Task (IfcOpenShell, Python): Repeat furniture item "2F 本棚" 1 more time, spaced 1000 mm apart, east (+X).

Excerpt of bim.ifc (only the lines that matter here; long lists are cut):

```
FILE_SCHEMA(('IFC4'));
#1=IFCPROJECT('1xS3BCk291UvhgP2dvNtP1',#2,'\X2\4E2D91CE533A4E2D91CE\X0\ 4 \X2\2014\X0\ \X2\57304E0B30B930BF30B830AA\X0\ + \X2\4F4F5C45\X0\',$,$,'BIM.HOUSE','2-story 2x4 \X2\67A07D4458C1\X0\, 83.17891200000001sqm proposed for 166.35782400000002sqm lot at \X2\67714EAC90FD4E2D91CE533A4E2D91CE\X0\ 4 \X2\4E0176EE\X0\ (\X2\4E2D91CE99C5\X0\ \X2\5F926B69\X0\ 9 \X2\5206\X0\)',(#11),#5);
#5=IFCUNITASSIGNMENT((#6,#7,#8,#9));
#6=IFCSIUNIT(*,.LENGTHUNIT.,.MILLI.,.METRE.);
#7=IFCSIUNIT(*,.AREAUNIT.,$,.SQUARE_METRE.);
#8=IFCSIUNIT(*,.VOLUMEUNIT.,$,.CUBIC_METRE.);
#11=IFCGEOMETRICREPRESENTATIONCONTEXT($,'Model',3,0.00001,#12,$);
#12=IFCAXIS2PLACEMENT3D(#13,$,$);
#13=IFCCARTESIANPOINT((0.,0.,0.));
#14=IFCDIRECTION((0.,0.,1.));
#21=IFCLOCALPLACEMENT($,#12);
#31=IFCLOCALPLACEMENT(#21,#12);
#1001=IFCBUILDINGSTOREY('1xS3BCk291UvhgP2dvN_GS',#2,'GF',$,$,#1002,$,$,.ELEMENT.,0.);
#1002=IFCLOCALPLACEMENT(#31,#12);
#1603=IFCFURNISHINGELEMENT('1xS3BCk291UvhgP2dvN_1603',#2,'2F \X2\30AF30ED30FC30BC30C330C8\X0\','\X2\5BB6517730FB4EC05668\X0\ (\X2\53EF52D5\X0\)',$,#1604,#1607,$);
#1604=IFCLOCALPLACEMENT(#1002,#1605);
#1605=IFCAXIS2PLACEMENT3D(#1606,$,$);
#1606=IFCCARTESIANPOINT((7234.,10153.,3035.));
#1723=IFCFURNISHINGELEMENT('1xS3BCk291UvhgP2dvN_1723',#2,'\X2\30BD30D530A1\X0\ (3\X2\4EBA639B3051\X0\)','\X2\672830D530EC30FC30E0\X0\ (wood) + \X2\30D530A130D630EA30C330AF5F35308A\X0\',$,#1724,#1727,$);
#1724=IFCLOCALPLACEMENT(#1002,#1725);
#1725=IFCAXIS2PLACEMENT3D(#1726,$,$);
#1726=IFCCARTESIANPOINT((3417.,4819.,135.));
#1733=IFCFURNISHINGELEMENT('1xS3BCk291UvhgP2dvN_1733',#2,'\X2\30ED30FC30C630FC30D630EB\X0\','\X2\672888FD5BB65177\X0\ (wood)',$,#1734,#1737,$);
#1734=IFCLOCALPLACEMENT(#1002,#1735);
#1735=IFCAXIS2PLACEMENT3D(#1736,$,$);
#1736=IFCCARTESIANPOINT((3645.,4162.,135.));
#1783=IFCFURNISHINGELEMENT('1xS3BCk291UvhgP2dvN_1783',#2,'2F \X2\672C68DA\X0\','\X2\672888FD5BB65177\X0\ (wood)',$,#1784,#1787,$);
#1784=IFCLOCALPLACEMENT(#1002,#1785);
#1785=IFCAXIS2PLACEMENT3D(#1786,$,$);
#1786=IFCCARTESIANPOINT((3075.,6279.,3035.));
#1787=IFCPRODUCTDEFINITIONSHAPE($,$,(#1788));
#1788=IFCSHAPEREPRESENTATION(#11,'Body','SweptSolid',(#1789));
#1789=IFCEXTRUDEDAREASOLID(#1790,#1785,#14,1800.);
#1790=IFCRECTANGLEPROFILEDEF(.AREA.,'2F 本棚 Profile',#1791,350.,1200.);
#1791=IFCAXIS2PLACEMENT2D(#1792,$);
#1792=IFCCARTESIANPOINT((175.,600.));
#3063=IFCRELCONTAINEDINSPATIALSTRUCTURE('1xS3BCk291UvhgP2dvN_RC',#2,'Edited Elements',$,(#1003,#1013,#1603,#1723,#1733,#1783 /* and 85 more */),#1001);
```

```python
import numpy as np
import ifcopenshell
import ifcopenshell.api.geometry
import ifcopenshell.api.root
import ifcopenshell.util.element
import ifcopenshell.util.placement
import ifcopenshell.util.unit

model = ifcopenshell.open("bim.ifc")
unit_scale = ifcopenshell.util.unit.calculate_unit_scale(model)


def reuse_history(source, copy):
    """copy_class also copies each property set's owner history, people and application; keep the originals."""
    for rel in copy.IsDefinedBy:
        if rel.is_a("IfcRelDefinesByProperties") and (history := rel.RelatingPropertyDefinition.OwnerHistory):
            rel.RelatingPropertyDefinition.OwnerHistory = source.OwnerHistory
            ifcopenshell.util.element.remove_deep2(model, history)


source = model.by_id(1783)
base = ifcopenshell.util.placement.get_local_placement(source.ObjectPlacement)
step = np.array([1.0, 0.0, 0.0]) * 1 / unit_scale

for i in range(1, 2):
    copy = ifcopenshell.api.root.copy_class(model, product=source)
    copy.Representation = ifcopenshell.util.element.copy_deep(
        model, source.Representation, exclude=["IfcGeometricRepresentationContext", "IfcRepresentationMap"]
    )
    reuse_history(source, copy)
    matrix = base.copy()
    matrix[:3, 3] += i * step
    print("added at", matrix[:3, 3].round(3) + 0.0)
    ifcopenshell.api.geometry.edit_object_placement(model, product=copy, matrix=matrix, is_si=False)

model.write("bim_edited.ifc")
```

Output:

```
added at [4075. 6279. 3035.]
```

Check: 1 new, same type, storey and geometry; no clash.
